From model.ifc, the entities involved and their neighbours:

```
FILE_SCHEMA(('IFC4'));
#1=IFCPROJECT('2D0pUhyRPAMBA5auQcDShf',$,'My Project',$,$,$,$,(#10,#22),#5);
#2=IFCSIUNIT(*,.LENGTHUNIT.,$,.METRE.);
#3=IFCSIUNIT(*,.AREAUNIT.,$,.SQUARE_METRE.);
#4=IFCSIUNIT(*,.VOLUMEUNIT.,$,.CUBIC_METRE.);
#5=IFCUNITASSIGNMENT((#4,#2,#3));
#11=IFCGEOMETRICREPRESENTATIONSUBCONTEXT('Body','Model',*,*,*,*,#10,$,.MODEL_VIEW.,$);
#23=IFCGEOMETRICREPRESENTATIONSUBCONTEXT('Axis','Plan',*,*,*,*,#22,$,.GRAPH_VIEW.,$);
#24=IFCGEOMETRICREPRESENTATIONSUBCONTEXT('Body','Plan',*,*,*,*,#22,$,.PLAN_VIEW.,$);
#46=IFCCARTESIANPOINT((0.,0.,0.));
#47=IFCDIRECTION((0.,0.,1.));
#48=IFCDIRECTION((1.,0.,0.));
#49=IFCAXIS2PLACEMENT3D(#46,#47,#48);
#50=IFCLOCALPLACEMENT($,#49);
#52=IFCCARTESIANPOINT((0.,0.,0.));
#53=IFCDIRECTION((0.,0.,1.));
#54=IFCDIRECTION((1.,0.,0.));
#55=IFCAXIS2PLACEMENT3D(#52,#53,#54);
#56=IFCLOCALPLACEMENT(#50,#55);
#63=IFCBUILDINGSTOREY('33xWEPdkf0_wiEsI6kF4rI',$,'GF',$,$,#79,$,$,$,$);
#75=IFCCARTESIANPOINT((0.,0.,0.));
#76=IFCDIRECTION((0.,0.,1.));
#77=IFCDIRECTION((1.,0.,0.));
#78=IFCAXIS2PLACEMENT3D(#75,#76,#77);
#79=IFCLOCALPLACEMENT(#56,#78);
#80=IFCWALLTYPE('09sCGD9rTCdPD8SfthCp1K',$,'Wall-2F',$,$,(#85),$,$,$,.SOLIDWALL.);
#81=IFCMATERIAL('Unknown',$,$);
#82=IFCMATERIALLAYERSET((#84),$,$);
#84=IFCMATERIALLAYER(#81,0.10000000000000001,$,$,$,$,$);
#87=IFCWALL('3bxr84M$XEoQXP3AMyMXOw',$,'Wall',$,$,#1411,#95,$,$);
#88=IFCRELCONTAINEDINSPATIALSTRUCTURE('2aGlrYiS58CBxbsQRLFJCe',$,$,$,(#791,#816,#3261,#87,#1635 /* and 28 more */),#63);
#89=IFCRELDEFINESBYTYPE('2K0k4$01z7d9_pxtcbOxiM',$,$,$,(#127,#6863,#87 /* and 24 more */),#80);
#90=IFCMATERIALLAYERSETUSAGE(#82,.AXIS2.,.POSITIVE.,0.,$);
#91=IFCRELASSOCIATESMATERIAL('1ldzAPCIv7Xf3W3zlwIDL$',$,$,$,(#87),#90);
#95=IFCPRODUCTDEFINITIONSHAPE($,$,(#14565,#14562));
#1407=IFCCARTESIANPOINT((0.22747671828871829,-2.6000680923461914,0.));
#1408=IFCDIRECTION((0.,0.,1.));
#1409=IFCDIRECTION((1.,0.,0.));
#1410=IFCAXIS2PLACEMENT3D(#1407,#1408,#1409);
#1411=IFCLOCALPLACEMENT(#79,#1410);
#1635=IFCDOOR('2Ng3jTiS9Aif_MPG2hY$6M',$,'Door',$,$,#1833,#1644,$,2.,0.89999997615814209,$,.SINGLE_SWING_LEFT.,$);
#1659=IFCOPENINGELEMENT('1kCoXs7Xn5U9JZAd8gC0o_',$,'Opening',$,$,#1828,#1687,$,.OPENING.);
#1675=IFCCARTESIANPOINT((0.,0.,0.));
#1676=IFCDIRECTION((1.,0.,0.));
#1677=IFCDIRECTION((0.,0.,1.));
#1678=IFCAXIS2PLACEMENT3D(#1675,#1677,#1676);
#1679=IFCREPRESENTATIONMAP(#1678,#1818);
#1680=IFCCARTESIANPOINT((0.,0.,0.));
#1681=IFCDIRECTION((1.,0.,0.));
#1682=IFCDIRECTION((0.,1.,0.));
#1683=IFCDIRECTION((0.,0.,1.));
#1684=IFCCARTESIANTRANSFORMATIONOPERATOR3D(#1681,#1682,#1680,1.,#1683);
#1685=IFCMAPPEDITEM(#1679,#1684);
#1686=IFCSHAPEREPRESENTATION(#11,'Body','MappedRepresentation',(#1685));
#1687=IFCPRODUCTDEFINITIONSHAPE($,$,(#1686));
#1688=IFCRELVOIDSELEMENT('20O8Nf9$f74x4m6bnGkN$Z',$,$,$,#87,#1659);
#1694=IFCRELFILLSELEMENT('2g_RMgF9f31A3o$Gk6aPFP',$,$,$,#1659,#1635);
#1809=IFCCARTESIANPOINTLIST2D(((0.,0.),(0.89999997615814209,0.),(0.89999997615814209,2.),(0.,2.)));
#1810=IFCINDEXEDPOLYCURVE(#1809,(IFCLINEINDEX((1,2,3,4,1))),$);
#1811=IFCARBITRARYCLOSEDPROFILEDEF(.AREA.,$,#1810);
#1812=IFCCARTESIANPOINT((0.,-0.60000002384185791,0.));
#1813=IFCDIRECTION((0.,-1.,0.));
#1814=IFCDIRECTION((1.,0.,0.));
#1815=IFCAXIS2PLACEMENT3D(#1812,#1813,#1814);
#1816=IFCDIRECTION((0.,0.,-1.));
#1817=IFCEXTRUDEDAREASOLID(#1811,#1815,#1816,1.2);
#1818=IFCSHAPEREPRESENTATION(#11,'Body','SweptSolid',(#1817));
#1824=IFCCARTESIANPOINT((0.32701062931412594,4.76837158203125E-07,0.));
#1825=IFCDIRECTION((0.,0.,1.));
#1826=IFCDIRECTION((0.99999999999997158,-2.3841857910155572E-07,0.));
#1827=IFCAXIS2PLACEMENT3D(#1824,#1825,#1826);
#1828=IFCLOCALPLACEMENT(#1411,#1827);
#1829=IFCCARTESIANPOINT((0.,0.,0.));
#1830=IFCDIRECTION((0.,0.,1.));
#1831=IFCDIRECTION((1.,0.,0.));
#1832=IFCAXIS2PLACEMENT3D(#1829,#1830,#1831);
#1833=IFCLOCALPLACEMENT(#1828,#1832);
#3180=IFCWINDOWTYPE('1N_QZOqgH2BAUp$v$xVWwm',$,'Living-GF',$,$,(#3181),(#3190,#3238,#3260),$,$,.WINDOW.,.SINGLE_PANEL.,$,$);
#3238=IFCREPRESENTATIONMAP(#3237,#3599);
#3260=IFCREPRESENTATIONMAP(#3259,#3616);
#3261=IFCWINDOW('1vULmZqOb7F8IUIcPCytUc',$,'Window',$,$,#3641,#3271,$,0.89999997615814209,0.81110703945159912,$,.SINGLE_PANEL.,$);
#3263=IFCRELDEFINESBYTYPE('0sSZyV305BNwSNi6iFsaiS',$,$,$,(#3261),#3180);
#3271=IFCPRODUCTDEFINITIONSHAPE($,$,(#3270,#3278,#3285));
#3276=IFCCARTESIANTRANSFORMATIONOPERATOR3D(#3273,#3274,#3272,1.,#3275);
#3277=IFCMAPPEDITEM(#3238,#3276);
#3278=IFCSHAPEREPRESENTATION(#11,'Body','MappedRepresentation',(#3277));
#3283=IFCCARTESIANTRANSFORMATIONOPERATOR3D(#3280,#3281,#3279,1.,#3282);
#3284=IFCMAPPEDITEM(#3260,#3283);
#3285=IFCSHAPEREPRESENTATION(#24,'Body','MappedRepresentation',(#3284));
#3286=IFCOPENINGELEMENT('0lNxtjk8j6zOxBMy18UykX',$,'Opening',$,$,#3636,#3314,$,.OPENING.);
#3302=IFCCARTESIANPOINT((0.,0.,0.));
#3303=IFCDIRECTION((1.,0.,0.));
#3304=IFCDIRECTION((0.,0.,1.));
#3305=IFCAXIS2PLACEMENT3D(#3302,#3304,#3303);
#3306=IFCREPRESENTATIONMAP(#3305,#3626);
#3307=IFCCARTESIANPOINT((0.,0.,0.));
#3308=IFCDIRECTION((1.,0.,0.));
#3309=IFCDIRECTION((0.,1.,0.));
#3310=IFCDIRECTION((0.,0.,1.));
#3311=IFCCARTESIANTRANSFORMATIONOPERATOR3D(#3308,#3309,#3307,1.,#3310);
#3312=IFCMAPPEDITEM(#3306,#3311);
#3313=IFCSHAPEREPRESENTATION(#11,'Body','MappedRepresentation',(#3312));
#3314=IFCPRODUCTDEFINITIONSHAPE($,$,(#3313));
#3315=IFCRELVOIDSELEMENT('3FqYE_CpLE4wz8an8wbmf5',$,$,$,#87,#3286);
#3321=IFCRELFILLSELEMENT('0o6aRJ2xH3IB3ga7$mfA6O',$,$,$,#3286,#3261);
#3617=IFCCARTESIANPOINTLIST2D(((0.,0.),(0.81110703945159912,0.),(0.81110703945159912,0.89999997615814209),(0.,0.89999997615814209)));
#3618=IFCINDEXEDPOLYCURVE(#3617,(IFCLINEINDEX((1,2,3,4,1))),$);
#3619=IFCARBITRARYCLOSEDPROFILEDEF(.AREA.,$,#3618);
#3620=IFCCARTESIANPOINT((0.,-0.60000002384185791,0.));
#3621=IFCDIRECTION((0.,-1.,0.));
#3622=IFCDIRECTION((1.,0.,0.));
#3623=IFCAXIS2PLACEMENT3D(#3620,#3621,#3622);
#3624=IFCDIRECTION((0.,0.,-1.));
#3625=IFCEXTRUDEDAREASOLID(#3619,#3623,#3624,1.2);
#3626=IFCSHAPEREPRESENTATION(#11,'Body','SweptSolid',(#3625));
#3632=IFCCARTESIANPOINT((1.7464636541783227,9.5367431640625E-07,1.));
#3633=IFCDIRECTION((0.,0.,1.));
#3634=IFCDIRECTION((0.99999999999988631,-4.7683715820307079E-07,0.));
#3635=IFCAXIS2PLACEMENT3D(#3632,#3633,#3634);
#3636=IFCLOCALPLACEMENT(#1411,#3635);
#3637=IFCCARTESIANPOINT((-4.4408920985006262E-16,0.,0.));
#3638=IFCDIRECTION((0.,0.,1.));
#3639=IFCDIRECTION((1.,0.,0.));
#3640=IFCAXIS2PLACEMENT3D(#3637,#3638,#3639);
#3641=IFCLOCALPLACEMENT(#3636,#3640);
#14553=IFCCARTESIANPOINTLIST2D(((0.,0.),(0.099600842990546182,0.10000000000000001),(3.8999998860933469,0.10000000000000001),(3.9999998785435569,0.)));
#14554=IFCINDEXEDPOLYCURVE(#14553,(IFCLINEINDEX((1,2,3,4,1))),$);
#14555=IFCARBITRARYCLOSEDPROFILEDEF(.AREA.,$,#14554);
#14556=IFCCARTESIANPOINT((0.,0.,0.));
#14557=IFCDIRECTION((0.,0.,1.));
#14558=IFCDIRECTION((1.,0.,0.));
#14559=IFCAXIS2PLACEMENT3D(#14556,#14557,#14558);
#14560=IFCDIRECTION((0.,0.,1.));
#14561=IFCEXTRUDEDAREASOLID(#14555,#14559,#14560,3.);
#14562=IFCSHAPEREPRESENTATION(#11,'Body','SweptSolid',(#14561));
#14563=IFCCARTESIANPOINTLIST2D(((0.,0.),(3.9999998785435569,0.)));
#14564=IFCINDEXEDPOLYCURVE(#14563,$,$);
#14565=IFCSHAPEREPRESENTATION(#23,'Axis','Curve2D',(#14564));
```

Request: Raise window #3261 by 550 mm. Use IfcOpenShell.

```python
import numpy as np
import ifcopenshell
import ifcopenshell.api.geometry
import ifcopenshell.util.placement
import ifcopenshell.util.unit

model = ifcopenshell.open("model.ifc")
unit_scale = ifcopenshell.util.unit.calculate_unit_scale(model)

window = model.by_guid("1vULmZqOb7F8IUIcPCytUc")
opening = window.FillsVoids[0].RelatingOpeningElement
dz = 0.55

shift = np.array([0.0, 0.0, dz])
# The window is placed relative to its opening, so it follows when the opening moves.
matrix = ifcopenshell.util.placement.get_local_placement(opening.ObjectPlacement)
matrix[:3, 3] += shift
ifcopenshell.api.geometry.edit_object_placement(
    model, product=opening, matrix=matrix, is_si=False, should_transform_children=True
)

print(f"moved by {dz * unit_scale:+.3f} m")

model.write("model_edited.ifc")
```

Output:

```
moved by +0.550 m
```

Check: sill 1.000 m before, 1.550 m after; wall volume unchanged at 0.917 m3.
